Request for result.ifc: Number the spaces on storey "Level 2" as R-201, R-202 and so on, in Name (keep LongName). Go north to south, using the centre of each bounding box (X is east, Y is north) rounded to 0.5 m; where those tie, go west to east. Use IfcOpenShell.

First a look at what the model holds.

```python
import ifcopenshell
import ifcopenshell.util.element
import ifcopenshell.util.placement

model = ifcopenshell.open("result.ifc")
print(model.schema)
storey = next(s for s in model.by_type("IfcBuildingStorey") if s.Name == "Level 2")
spaces = [e for e in ifcopenshell.util.element.get_decomposition(storey) if e.is_a("IfcSpace")]
for e in sorted(spaces, key=lambda e: e.id()):
    origin = ifcopenshell.util.placement.get_local_placement(e.ObjectPlacement)[:3, 3]
    print(e.id(), e.Name, e.LongName, origin.round(2) + 0.0, sep=" | ")
```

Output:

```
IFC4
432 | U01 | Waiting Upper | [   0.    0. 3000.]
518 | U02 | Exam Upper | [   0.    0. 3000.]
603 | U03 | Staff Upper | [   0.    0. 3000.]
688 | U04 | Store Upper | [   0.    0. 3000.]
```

```python
import ifcopenshell
import ifcopenshell.geom
import ifcopenshell.util.element
import ifcopenshell.util.shape

model = ifcopenshell.open("result.ifc")
settings = ifcopenshell.geom.settings()
settings.set("use-world-coords", True)


def centre(element):
    shape = ifcopenshell.geom.create_shape(settings, element)
    return ifcopenshell.util.shape.get_bbox_centroid(shape.geometry)


storey = next(s for s in model.by_type("IfcBuildingStorey") if s.Name == "Level 2")
spaces = [e for e in ifcopenshell.util.element.get_decomposition(storey) if e.is_a("IfcSpace")]

# Insertion points can sit at a corner or the storey origin, so sort by the geometry (in metres).
centres = {e: centre(e) for e in spaces}
spaces.sort(key=lambda e: (-round(centres[e][1] / 0.5), centres[e][0]))

for i, e in enumerate(spaces, start=1):
    number = f"R-2{i:02d}"
    e.Name = number
    print(e.id(), number)

model.write("result-out.ifc")
```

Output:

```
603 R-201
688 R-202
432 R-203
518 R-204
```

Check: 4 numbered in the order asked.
